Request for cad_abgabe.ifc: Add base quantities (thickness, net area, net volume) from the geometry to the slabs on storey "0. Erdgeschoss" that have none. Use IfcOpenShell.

First a look at what the model holds.

```python
import ifcopenshell
import ifcopenshell.util.element
import ifcopenshell.util.unit

model = ifcopenshell.open("cad_abgabe.ifc")
print(model.schema)
for unit_type in ("LENGTHUNIT", "AREAUNIT", "VOLUMEUNIT"):
    print(unit_type, ifcopenshell.util.unit.calculate_unit_scale(model, unit_type))
storey = next(s for s in model.by_type("IfcBuildingStorey") if s.Name == "0. Erdgeschoss")
slabs = [e for e in ifcopenshell.util.element.get_decomposition(storey) if e.is_a("IfcSlab")]
for e in sorted(slabs, key=lambda e: e.id()):
    print(e.id(), e.is_a(), e.Name, list(ifcopenshell.util.element.get_psets(e, qtos_only=True)), sep=" | ")
```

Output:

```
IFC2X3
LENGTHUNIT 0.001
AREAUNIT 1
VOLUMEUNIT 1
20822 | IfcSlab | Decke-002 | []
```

```python
import ifcopenshell
import ifcopenshell.api.pset
import ifcopenshell.geom
import ifcopenshell.util.element
import ifcopenshell.util.shape
import ifcopenshell.util.unit

model = ifcopenshell.open("cad_abgabe.ifc")
unit_scale = ifcopenshell.util.unit.calculate_unit_scale(model)
area_scale = ifcopenshell.util.unit.calculate_unit_scale(model, "AREAUNIT")
volume_scale = ifcopenshell.util.unit.calculate_unit_scale(model, "VOLUMEUNIT")
settings = ifcopenshell.geom.settings()

storey = next(s for s in model.by_type("IfcBuildingStorey") if s.Name == "0. Erdgeschoss")
slabs = [e for e in ifcopenshell.util.element.get_decomposition(storey) if e.is_a("IfcSlab")]

for e in sorted(slabs, key=lambda e: e.id()):
    if ifcopenshell.util.element.get_psets(e, qtos_only=True, should_inherit=False):
        continue
    # Geometry comes back in metres, in the element's own axes.
    shape = ifcopenshell.geom.create_shape(settings, e)
    values = {
        "Width": ifcopenshell.util.shape.get_z(shape.geometry) / unit_scale,
        "NetArea": ifcopenshell.util.shape.get_footprint_area(shape.geometry) / area_scale,
        "NetVolume": ifcopenshell.util.shape.get_volume(shape.geometry) / volume_scale,
    }
    qto = ifcopenshell.api.pset.add_qto(model, product=e, name="BaseQuantities")
    ifcopenshell.api.pset.edit_qto(model, qto=qto, properties=values)
    print(e.id(), {k: round(v, 3) for k, v in values.items()})

model.write("cad_abgabe_rev.ifc")
```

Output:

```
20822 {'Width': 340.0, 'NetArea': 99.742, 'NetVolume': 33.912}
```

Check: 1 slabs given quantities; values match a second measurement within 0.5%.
